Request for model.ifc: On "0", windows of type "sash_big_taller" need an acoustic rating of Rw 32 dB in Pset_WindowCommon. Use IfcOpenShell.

First a look at what the model holds.

```python
import ifcopenshell
import ifcopenshell.util.element

model = ifcopenshell.open("model.ifc")
print(model.schema)
storey = next(s for s in model.by_type("IfcBuildingStorey") if s.Name == "0")
windows = [e for e in ifcopenshell.util.element.get_decomposition(storey) if e.is_a("IfcWindow")]
seen = {}
for e in windows:
    element_type = ifcopenshell.util.element.get_type(e)
    key = (element_type.Name if element_type != e and element_type else None, ifcopenshell.util.element.get_pset(e, "Pset_WindowCommon", "AcousticRating"))
    seen[key] = seen.get(key, 0) + 1
for (name, value), count in sorted(seen.items(), key=str):
    print(count, "x", name, "|", value)
```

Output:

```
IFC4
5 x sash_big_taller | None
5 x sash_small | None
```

```python
import ifcopenshell
import ifcopenshell.api.pset
import ifcopenshell.util.element

model = ifcopenshell.open("model.ifc")

storey = next(s for s in model.by_type("IfcBuildingStorey") if s.Name == "0")
windows = [e for e in ifcopenshell.util.element.get_decomposition(storey) if e.is_a("IfcWindow")]

count = 0
for e in windows:
    element_type = ifcopenshell.util.element.get_type(e)
    if element_type in (None, e) or element_type.Name != "sash_big_taller":
        continue
    # add_pset returns the element's existing set when there is one.
    pset = ifcopenshell.api.pset.add_pset(model, product=e, name="Pset_WindowCommon")
    ifcopenshell.api.pset.edit_pset(model, pset=pset, properties={"AcousticRating": "Rw 32 dB"})
    count += 1

print(count, "windows updated")

model.write("model_v2.ifc")
```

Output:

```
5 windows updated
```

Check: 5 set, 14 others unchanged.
